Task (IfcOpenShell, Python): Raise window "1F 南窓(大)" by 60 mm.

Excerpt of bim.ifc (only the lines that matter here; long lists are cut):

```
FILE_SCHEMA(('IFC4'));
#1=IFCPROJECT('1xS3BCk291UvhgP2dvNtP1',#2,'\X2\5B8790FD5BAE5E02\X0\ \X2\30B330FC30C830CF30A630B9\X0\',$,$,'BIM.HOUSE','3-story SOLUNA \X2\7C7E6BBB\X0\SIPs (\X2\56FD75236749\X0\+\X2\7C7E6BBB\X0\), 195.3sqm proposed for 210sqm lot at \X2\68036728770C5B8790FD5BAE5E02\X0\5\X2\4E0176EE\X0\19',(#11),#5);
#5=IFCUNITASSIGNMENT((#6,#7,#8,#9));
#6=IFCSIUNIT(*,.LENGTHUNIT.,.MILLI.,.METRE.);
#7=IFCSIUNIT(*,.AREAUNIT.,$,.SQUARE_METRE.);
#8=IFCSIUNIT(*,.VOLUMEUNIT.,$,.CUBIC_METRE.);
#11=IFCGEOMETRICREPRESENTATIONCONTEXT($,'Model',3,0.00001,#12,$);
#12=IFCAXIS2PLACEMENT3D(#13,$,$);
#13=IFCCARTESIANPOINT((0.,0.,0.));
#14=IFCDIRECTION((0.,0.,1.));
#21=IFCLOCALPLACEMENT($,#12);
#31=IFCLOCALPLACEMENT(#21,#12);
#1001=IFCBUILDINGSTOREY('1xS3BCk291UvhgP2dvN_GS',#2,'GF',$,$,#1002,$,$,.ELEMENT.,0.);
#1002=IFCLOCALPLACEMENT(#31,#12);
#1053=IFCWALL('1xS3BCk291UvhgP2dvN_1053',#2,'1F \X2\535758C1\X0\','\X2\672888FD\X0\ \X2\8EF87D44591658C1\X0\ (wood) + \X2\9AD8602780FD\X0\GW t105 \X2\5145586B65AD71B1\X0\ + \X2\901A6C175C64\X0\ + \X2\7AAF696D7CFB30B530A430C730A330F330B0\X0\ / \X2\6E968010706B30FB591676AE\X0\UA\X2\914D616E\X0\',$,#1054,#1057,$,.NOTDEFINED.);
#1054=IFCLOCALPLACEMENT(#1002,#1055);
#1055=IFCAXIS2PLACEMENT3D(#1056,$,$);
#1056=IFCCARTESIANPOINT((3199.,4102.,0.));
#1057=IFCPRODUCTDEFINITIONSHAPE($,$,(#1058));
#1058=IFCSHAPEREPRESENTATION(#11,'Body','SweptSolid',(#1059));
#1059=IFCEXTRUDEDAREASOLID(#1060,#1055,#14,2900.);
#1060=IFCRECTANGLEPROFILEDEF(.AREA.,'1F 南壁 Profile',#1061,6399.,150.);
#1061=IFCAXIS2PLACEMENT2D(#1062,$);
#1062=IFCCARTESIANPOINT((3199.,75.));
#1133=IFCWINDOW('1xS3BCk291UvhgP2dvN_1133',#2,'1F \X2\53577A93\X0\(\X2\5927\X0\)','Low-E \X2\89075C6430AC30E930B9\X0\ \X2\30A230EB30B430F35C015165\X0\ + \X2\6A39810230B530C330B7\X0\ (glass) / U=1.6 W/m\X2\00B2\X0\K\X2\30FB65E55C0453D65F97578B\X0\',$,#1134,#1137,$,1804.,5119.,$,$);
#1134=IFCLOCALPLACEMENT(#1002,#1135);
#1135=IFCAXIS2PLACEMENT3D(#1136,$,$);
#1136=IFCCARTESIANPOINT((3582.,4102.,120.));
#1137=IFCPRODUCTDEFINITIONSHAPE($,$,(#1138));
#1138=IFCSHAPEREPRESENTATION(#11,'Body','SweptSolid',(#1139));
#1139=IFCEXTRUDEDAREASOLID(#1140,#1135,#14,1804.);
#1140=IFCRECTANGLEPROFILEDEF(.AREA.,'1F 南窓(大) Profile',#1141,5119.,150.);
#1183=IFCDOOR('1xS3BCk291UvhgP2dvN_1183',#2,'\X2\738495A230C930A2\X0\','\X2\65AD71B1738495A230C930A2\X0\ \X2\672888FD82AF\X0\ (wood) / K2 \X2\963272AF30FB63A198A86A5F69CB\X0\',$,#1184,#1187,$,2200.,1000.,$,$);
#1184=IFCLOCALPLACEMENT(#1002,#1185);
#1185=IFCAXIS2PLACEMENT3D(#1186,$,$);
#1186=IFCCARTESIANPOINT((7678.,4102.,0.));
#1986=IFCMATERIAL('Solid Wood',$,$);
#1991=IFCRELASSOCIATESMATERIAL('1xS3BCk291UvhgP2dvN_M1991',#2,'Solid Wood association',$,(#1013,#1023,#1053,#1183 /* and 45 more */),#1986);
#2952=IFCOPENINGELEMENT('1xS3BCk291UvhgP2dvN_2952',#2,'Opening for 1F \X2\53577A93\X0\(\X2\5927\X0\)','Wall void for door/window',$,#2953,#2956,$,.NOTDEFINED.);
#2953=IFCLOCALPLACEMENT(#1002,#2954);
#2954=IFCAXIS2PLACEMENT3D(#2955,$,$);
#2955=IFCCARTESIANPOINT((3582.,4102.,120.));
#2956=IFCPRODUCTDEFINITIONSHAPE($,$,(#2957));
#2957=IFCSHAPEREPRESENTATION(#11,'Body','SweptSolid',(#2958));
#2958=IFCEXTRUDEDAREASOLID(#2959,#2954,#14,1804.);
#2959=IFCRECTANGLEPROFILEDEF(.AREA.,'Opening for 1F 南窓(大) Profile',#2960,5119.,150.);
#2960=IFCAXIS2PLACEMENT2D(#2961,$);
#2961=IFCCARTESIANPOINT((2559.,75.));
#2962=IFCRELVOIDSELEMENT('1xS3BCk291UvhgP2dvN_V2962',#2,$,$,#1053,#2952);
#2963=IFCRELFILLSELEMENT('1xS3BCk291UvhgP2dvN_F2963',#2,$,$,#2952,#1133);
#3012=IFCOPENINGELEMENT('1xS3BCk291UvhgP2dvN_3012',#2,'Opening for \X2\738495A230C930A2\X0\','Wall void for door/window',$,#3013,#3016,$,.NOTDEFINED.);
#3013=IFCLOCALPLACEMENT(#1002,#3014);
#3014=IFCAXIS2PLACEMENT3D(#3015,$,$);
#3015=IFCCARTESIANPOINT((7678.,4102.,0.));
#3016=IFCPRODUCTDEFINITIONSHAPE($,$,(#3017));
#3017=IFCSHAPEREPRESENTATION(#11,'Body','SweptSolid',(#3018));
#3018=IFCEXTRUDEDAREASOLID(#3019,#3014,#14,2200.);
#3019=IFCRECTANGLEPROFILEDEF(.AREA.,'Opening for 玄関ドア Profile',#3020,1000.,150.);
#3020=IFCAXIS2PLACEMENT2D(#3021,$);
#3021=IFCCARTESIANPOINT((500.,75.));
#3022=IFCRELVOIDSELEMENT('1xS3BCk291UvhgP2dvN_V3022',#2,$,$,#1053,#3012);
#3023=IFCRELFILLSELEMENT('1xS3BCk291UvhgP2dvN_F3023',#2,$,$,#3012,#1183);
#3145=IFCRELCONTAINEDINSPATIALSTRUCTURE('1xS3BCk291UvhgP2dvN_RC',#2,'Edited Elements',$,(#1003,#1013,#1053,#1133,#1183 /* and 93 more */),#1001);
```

```python
import numpy as np
import ifcopenshell
import ifcopenshell.api.geometry
import ifcopenshell.util.placement
import ifcopenshell.util.unit

model = ifcopenshell.open("bim.ifc")
unit_scale = ifcopenshell.util.unit.calculate_unit_scale(model)

window = model.by_guid("1xS3BCk291UvhgP2dvN_1133")
opening = window.FillsVoids[0].RelatingOpeningElement
dz = 0.06 / unit_scale

shift = np.array([0.0, 0.0, dz])
# The window is not placed relative to its opening, so move both.
for product in (opening, window):
    matrix = ifcopenshell.util.placement.get_local_placement(product.ObjectPlacement)
    matrix[:3, 3] += shift
    ifcopenshell.api.geometry.edit_object_placement(model, product=product, matrix=matrix, is_si=False)

print(f"moved by {dz * unit_scale:+.3f} m")

model.write("bim_rev.ifc")
```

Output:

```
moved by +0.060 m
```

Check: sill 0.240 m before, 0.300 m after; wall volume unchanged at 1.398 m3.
